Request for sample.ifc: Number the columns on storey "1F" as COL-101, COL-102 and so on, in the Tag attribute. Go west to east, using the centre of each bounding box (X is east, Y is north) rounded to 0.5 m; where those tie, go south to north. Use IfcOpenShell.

First a look at what the model holds.

```python
import ifcopenshell
import ifcopenshell.util.element
import ifcopenshell.util.placement

model = ifcopenshell.open("sample.ifc")
print(model.schema)
storey = next(s for s in model.by_type("IfcBuildingStorey") if s.Name == "1F")
columns = [e for e in ifcopenshell.util.element.get_decomposition(storey) if e.is_a("IfcColumn")]
for e in sorted(columns, key=lambda e: e.id()):
    origin = ifcopenshell.util.placement.get_local_placement(e.ObjectPlacement)[:3, 3]
    print(e.id(), e.Tag, e.Name, origin.round(2) + 0.0, sep=" | ")
```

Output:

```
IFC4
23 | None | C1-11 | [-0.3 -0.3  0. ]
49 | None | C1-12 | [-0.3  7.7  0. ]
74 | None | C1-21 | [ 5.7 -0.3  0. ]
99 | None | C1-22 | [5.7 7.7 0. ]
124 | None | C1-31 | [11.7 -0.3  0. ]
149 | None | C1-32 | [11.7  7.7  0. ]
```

```python
import ifcopenshell
import ifcopenshell.geom
import ifcopenshell.util.element
import ifcopenshell.util.shape

model = ifcopenshell.open("sample.ifc")
settings = ifcopenshell.geom.settings()
settings.set("use-world-coords", True)


def centre(element):
    shape = ifcopenshell.geom.create_shape(settings, element)
    return ifcopenshell.util.shape.get_bbox_centroid(shape.geometry)


storey = next(s for s in model.by_type("IfcBuildingStorey") if s.Name == "1F")
columns = [e for e in ifcopenshell.util.element.get_decomposition(storey) if e.is_a("IfcColumn")]

# Insertion points can sit at a corner or the storey origin, so sort by the geometry (in metres).
centres = {e: centre(e) for e in columns}
columns.sort(key=lambda e: (round(centres[e][0] / 0.5), centres[e][1]))

for i, e in enumerate(columns, start=1):
    number = f"COL-1{i:02d}"
    e.Tag = number
    print(e.id(), number)

model.write("sample_v2.ifc")
```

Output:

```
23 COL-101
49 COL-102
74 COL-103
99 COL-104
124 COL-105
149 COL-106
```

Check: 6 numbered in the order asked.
